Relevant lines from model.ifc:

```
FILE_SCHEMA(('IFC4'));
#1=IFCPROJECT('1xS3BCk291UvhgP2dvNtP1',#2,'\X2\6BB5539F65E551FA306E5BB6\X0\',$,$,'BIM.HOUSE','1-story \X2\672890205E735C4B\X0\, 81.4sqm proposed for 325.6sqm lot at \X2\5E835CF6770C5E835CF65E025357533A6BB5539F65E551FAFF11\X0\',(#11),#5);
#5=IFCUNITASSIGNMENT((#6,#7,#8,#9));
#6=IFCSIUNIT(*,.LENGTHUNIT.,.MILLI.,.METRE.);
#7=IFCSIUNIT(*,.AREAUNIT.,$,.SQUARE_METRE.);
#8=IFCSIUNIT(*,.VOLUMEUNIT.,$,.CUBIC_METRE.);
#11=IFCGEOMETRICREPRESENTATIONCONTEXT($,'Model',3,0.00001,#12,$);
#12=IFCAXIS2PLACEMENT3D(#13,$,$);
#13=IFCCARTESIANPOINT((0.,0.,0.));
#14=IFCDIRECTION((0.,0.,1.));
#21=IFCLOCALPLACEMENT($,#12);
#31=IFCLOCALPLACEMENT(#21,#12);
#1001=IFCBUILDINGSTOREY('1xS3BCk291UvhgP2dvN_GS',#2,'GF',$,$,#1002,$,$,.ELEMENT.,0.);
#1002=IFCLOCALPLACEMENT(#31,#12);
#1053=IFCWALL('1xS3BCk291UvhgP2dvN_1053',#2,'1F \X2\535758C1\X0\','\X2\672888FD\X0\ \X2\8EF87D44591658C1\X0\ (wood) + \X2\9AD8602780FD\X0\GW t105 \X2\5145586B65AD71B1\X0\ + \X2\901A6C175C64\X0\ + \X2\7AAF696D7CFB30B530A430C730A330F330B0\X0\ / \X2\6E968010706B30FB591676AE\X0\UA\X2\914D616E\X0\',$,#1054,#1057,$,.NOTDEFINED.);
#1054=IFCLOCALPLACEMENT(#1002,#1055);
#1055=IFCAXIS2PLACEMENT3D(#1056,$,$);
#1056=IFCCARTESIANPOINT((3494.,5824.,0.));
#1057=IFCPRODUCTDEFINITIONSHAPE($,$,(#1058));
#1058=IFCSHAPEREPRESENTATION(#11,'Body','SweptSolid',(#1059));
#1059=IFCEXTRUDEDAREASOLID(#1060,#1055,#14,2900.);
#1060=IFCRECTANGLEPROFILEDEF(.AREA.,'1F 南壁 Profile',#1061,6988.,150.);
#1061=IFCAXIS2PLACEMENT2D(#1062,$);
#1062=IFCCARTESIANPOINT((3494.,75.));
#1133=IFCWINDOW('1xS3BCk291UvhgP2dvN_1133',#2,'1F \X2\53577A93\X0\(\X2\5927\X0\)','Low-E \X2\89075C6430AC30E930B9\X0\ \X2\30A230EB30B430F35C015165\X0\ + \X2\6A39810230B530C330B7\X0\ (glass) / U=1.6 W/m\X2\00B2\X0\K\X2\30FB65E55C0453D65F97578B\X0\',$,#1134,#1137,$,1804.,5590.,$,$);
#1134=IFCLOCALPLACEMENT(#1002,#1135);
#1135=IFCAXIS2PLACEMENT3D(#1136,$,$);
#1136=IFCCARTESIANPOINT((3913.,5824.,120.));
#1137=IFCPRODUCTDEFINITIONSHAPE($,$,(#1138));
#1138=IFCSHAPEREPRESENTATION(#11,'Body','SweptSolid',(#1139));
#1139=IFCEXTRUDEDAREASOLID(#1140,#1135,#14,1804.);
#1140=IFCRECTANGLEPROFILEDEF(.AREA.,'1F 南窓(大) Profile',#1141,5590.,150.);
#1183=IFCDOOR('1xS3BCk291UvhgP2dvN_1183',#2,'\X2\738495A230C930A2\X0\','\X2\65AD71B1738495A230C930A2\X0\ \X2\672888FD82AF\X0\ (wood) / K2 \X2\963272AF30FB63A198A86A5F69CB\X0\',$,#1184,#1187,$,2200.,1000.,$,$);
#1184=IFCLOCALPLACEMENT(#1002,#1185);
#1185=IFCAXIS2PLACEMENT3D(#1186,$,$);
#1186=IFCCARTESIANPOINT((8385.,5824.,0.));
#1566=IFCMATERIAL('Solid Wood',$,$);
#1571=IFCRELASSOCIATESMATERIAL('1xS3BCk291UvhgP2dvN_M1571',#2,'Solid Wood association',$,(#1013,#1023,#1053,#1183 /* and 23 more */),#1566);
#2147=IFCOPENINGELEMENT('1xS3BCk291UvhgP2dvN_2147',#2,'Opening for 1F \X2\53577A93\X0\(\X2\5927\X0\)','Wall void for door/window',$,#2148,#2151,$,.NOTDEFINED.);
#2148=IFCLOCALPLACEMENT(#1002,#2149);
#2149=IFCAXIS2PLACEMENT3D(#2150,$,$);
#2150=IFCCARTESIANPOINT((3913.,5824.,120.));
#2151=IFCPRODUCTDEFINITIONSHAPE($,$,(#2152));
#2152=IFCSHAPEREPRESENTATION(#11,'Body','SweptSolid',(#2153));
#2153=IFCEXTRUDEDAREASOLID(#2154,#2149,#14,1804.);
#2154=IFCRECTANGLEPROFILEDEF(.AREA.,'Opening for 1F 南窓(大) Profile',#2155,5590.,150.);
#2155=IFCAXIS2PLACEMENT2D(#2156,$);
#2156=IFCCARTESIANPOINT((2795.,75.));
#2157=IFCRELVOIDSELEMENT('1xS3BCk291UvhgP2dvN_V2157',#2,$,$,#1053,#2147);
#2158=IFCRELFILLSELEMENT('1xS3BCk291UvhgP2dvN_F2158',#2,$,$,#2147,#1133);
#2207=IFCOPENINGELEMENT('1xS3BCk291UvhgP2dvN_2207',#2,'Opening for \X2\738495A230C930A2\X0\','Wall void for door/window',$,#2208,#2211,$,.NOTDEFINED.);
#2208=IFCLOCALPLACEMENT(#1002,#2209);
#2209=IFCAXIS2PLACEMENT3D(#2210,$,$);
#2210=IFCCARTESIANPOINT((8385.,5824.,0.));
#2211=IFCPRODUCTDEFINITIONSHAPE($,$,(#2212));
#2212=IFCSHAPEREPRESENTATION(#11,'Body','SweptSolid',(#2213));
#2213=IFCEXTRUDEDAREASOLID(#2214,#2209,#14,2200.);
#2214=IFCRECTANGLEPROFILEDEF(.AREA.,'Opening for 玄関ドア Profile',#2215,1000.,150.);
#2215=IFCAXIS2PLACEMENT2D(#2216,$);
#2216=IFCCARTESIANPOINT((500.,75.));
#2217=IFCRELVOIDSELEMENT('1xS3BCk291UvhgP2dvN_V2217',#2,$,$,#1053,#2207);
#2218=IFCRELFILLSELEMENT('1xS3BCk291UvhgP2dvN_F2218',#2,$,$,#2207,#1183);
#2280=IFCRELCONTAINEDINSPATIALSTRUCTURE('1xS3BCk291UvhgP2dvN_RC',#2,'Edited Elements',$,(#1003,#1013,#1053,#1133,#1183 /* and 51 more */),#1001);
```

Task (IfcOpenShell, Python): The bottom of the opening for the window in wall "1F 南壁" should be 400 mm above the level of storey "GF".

```python
import numpy as np
import ifcopenshell
import ifcopenshell.api.geometry
import ifcopenshell.geom
import ifcopenshell.util.element
import ifcopenshell.util.placement
import ifcopenshell.util.shape
import ifcopenshell.util.unit

model = ifcopenshell.open("model.ifc")
unit_scale = ifcopenshell.util.unit.calculate_unit_scale(model)

window = model.by_guid("1xS3BCk291UvhgP2dvN_1133")
opening = window.FillsVoids[0].RelatingOpeningElement
storey = ifcopenshell.util.element.get_container(window, ifc_class="IfcBuildingStorey")
level = ifcopenshell.util.placement.get_local_placement(storey.ObjectPlacement)[2, 3]

# The opening's origin need not be at the sill, so measure its lowest point.
shape = ifcopenshell.geom.create_shape(ifcopenshell.geom.settings(), opening)
bottom = ifcopenshell.util.shape.get_shape_bottom_elevation(shape, shape.geometry) / unit_scale
dz = level + 400.0 - bottom

shift = np.array([0.0, 0.0, dz])
# The window is not placed relative to its opening, so move both.
for product in (opening, window):
    matrix = ifcopenshell.util.placement.get_local_placement(product.ObjectPlacement)
    matrix[:3, 3] += shift
    ifcopenshell.api.geometry.edit_object_placement(model, product=product, matrix=matrix, is_si=False)

print(f"moved by {dz * unit_scale:+.3f} m")

model.write("model_rev.ifc")
```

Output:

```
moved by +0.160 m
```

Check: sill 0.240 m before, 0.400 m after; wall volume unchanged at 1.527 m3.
